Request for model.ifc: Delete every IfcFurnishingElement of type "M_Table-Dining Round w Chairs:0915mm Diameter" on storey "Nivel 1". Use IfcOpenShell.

First a look at what the model holds.

```python
import ifcopenshell
import ifcopenshell.util.element

model = ifcopenshell.open("model.ifc")
print(model.schema)
storey = next(s for s in model.by_type("IfcBuildingStorey") if s.Name == "Nivel 1")
furniture = [e for e in ifcopenshell.util.element.get_decomposition(storey) if e.is_a("IfcFurnishingElement")]
seen = {}
for e in furniture:
    element_type = ifcopenshell.util.element.get_type(e)
    name = element_type.Name if element_type not in (None, e) else None
    seen[name] = seen.get(name, 0) + 1
for name, count in sorted(seen.items(), key=str):
    print(count, "x", name)
```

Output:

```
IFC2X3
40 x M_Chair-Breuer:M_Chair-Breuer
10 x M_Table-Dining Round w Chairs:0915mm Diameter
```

```python
import ifcopenshell
import ifcopenshell.api.root
import ifcopenshell.util.element

model = ifcopenshell.open("model.ifc")

storey = next(s for s in model.by_type("IfcBuildingStorey") if s.Name == "Nivel 1")
furniture = [e for e in ifcopenshell.util.element.get_decomposition(storey) if e.is_a("IfcFurnishingElement")]
targets = [e for e in furniture if (t := ifcopenshell.util.element.get_type(e)) not in (None, e) and t.Name == "M_Table-Dining Round w Chairs:0915mm Diameter"]

for e in targets:
    ifcopenshell.api.root.remove_product(model, product=e)
print(len(targets), "removed")

model.write("model_updated.ifc")
```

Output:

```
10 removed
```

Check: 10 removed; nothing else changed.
